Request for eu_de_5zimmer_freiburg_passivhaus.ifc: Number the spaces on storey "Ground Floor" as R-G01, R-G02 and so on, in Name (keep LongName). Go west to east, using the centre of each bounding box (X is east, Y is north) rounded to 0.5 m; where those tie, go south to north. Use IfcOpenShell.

First a look at what the model holds.

```python
import ifcopenshell
import ifcopenshell.util.element
import ifcopenshell.util.placement

model = ifcopenshell.open("eu_de_5zimmer_freiburg_passivhaus.ifc")
print(model.schema)
storey = next(s for s in model.by_type("IfcBuildingStorey") if s.Name == "Ground Floor")
spaces = [e for e in ifcopenshell.util.element.get_decomposition(storey) if e.is_a("IfcSpace")]
for e in sorted(spaces, key=lambda e: e.id()):
    origin = ifcopenshell.util.placement.get_local_placement(e.ObjectPlacement)[:3, 3]
    print(e.id(), e.Name, e.LongName, origin.round(2) + 0.0, sep=" | ")
```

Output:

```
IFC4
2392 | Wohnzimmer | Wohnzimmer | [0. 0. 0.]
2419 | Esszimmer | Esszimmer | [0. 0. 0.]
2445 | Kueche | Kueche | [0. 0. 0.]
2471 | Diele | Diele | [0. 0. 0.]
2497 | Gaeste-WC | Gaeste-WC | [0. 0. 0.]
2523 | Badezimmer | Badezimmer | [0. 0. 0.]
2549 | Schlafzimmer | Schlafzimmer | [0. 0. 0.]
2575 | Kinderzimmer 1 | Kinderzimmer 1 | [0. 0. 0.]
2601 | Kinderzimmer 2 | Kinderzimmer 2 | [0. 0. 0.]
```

```python
import ifcopenshell
import ifcopenshell.geom
import ifcopenshell.util.element
import ifcopenshell.util.shape

model = ifcopenshell.open("eu_de_5zimmer_freiburg_passivhaus.ifc")
settings = ifcopenshell.geom.settings()
settings.set("use-world-coords", True)


def centre(element):
    shape = ifcopenshell.geom.create_shape(settings, element)
    return ifcopenshell.util.shape.get_bbox_centroid(shape.geometry)


storey = next(s for s in model.by_type("IfcBuildingStorey") if s.Name == "Ground Floor")
spaces = [e for e in ifcopenshell.util.element.get_decomposition(storey) if e.is_a("IfcSpace")]

# Insertion points can sit at a corner or the storey origin, so sort by the geometry (in metres).
centres = {e: centre(e) for e in spaces}
spaces.sort(key=lambda e: (round(centres[e][0] / 0.5), centres[e][1]))

for i, e in enumerate(spaces, start=1):
    number = f"R-G{i:02d}"
    e.Name = number
    print(e.id(), number)

model.write("eu_de_5zimmer_freiburg_passivhaus_v2.ifc")
```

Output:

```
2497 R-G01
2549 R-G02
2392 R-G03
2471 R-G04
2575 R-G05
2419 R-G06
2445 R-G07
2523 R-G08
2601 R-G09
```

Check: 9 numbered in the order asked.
